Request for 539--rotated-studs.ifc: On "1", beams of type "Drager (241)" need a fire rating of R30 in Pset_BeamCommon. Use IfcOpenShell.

First a look at what the model holds.

```python
import ifcopenshell
import ifcopenshell.util.element

model = ifcopenshell.open("539--rotated-studs.ifc")
print(model.schema)
storey = next(s for s in model.by_type("IfcBuildingStorey") if s.Name == "1")
beams = [e for e in ifcopenshell.util.element.get_decomposition(storey) if e.is_a("IfcBeam")]
seen = {}
for e in beams:
    element_type = ifcopenshell.util.element.get_type(e)
    key = (element_type.Name if element_type != e and element_type else None, ifcopenshell.util.element.get_pset(e, "Pset_BeamCommon", "FireRating"))
    seen[key] = seen.get(key, 0) + 1
for (name, value), count in sorted(seen.items(), key=str):
    print(count, "x", name, "|", value)
```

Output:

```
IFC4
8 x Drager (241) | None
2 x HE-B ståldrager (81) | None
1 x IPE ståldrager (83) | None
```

```python
import ifcopenshell
import ifcopenshell.api.pset
import ifcopenshell.util.element

model = ifcopenshell.open("539--rotated-studs.ifc")

storey = next(s for s in model.by_type("IfcBuildingStorey") if s.Name == "1")
beams = [e for e in ifcopenshell.util.element.get_decomposition(storey) if e.is_a("IfcBeam")]

count = 0
for e in beams:
    element_type = ifcopenshell.util.element.get_type(e)
    if element_type in (None, e) or element_type.Name != "Drager (241)":
        continue
    # add_pset returns the element's existing set when there is one.
    pset = ifcopenshell.api.pset.add_pset(model, product=e, name="Pset_BeamCommon")
    ifcopenshell.api.pset.edit_pset(model, pset=pset, properties={"FireRating": "R30"})
    count += 1

print(count, "beams updated")

model.write("539--rotated-studs_rev.ifc")
```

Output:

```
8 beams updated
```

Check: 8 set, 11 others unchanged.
